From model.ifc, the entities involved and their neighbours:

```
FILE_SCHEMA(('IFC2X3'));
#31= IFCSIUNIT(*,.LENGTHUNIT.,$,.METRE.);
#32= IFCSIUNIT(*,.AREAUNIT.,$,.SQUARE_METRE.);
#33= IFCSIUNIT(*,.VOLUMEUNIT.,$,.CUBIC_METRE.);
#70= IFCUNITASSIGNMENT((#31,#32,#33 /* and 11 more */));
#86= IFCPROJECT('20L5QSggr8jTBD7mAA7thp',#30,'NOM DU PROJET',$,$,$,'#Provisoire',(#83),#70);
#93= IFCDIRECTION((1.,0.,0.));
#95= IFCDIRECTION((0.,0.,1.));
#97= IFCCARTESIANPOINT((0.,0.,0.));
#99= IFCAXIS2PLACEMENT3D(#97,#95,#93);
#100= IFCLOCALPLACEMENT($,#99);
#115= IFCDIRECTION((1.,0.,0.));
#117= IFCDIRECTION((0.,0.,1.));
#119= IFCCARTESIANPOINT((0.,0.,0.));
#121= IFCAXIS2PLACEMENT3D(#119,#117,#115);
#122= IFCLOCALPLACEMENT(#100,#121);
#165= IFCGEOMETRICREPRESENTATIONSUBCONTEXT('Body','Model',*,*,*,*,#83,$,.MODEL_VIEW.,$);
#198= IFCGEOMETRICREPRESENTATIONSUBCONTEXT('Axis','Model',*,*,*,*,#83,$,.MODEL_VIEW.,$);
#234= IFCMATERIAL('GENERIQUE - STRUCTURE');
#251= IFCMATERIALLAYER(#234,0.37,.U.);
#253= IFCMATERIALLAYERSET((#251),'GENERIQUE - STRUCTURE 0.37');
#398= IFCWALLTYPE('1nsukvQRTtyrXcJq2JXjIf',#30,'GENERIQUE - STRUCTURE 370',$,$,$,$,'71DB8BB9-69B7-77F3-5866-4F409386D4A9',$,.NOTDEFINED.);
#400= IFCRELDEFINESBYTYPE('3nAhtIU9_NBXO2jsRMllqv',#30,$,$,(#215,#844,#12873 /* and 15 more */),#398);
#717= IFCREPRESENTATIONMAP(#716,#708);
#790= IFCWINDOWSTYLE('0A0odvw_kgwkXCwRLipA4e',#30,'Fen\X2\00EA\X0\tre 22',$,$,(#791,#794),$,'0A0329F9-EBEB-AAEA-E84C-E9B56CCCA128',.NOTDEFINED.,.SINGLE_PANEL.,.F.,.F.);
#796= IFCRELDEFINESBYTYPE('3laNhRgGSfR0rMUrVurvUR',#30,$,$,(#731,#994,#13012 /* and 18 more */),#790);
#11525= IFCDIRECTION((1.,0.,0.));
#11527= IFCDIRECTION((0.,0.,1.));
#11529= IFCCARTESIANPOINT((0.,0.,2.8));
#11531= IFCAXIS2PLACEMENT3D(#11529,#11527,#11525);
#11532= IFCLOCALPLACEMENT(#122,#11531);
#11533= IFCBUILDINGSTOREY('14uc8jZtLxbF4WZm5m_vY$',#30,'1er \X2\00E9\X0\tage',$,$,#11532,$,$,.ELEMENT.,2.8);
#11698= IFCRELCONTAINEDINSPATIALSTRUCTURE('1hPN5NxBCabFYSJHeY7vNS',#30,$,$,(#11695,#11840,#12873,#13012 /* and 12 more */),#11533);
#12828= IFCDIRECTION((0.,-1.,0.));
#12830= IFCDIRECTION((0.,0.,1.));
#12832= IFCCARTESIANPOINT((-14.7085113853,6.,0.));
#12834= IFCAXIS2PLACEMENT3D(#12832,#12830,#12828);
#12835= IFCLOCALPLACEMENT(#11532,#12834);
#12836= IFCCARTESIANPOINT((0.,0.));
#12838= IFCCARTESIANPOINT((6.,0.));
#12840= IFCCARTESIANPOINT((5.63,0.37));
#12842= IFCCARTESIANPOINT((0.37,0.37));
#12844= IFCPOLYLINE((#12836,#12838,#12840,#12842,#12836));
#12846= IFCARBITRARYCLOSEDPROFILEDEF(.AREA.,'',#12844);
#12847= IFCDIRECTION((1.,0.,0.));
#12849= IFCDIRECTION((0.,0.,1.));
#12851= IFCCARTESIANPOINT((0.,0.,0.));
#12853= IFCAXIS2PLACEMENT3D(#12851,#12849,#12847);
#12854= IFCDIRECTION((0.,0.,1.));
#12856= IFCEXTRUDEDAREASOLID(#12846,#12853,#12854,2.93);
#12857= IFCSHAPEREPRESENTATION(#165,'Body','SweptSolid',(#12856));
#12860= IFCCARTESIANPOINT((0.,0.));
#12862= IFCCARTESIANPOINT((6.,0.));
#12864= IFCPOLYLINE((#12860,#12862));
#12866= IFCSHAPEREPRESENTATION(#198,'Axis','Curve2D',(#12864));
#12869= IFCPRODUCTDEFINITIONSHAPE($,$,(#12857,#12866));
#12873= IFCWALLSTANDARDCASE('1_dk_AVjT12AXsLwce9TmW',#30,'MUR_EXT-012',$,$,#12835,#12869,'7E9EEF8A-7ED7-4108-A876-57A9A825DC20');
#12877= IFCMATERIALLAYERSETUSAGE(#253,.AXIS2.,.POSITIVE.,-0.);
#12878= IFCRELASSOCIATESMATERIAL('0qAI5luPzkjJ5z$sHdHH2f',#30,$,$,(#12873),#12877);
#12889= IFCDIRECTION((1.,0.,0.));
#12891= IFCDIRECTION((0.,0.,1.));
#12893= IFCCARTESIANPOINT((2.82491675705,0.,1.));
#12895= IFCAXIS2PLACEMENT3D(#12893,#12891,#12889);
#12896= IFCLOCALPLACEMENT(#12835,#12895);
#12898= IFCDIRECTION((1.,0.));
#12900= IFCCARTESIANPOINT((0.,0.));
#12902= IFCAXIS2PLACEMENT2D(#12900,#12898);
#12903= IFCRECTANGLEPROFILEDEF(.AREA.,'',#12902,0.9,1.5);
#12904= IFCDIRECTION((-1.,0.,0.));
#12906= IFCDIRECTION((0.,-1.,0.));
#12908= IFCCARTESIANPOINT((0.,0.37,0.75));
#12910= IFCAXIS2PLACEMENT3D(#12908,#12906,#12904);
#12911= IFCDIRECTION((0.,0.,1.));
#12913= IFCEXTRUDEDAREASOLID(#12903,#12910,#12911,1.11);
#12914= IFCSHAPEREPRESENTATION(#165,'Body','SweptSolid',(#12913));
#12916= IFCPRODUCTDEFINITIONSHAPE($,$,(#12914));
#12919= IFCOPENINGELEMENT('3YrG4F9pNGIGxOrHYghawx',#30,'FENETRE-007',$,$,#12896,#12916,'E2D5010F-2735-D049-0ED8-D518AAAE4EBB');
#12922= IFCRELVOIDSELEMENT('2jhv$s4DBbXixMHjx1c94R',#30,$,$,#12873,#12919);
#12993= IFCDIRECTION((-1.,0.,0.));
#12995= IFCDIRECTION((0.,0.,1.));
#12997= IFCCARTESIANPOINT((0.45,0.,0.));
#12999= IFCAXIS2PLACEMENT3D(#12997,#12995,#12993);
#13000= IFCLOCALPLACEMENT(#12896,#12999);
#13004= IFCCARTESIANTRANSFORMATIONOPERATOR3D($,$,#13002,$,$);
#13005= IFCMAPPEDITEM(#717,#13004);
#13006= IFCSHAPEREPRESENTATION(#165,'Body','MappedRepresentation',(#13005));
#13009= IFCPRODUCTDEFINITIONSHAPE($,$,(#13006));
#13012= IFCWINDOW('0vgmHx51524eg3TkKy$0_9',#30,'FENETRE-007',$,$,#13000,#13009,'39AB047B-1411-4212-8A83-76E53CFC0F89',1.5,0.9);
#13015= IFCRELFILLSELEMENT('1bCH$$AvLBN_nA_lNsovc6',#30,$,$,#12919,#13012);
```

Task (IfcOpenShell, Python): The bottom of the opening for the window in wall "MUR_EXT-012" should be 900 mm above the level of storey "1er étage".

```python
import numpy as np
import ifcopenshell
import ifcopenshell.api.geometry
import ifcopenshell.geom
import ifcopenshell.util.element
import ifcopenshell.util.placement
import ifcopenshell.util.shape
import ifcopenshell.util.unit

model = ifcopenshell.open("model.ifc")
unit_scale = ifcopenshell.util.unit.calculate_unit_scale(model)

window = model.by_guid("0vgmHx51524eg3TkKy$0_9")
opening = window.FillsVoids[0].RelatingOpeningElement
storey = ifcopenshell.util.element.get_container(window, ifc_class="IfcBuildingStorey")
level = ifcopenshell.util.placement.get_local_placement(storey.ObjectPlacement)[2, 3]

# The opening's origin need not be at the sill, so measure its lowest point.
shape = ifcopenshell.geom.create_shape(ifcopenshell.geom.settings(), opening)
bottom = ifcopenshell.util.shape.get_shape_bottom_elevation(shape, shape.geometry) / unit_scale
dz = level + 0.9 / unit_scale - bottom

shift = np.array([0.0, 0.0, dz])
# The window is placed relative to its opening, so it follows when the opening moves.
matrix = ifcopenshell.util.placement.get_local_placement(opening.ObjectPlacement)
matrix[:3, 3] += shift
ifcopenshell.api.geometry.edit_object_placement(
    model, product=opening, matrix=matrix, is_si=False, should_transform_children=True
)

print(f"moved by {dz * unit_scale:+.3f} m")

model.write("model_edited.ifc")
```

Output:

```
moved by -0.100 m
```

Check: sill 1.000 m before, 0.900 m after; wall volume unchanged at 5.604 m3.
